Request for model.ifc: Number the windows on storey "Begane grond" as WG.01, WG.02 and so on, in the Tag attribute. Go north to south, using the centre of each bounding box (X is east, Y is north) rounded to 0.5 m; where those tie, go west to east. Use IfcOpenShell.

First a look at what the model holds.

```python
import ifcopenshell
import ifcopenshell.util.element
import ifcopenshell.util.placement

model = ifcopenshell.open("model.ifc")
print(model.schema)
storey = next(s for s in model.by_type("IfcBuildingStorey") if s.Name == "Begane grond")
windows = [e for e in ifcopenshell.util.element.get_decomposition(storey) if e.is_a("IfcWindow")]
for e in sorted(windows, key=lambda e: e.id()):
    origin = ifcopenshell.util.placement.get_local_placement(e.ObjectPlacement)[:3, 3]
    print(e.id(), e.Tag, e.Name, origin.round(2) + 0.0, sep=" | ")
```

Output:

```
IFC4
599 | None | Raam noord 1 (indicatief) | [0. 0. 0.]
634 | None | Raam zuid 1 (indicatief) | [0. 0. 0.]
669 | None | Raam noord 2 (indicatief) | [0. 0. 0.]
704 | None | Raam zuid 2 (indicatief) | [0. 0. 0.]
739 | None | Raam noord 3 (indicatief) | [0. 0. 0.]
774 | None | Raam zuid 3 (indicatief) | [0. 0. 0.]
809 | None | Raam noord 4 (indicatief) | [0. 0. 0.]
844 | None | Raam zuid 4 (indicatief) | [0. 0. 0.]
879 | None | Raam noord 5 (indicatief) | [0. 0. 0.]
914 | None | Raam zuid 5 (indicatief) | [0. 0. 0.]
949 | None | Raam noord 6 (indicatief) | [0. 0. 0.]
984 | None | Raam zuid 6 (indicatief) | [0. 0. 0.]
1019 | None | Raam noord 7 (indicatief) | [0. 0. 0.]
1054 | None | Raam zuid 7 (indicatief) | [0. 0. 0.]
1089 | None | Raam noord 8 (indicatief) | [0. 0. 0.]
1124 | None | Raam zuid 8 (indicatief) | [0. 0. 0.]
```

```python
import ifcopenshell
import ifcopenshell.geom
import ifcopenshell.util.element
import ifcopenshell.util.shape

model = ifcopenshell.open("model.ifc")
settings = ifcopenshell.geom.settings()
settings.set("use-world-coords", True)


def centre(element):
    shape = ifcopenshell.geom.create_shape(settings, element)
    return ifcopenshell.util.shape.get_bbox_centroid(shape.geometry)


storey = next(s for s in model.by_type("IfcBuildingStorey") if s.Name == "Begane grond")
windows = [e for e in ifcopenshell.util.element.get_decomposition(storey) if e.is_a("IfcWindow")]

# Insertion points can sit at a corner or the storey origin, so sort by the geometry (in metres).
centres = {e: centre(e) for e in windows}
windows.sort(key=lambda e: (-round(centres[e][1] / 0.5), centres[e][0]))

for i, e in enumerate(windows, start=1):
    number = f"WG.{i:02d}"
    e.Tag = number
    print(e.id(), number)

model.write("model_rev.ifc")
```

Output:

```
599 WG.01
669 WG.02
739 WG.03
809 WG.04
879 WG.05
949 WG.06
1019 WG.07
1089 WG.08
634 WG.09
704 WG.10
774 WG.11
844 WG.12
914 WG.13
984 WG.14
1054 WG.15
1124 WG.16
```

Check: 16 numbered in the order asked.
